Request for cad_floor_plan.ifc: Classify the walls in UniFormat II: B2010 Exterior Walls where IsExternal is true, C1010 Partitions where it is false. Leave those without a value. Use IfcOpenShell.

First a look at what the model holds.

```python
import ifcopenshell
import ifcopenshell.util.element

model = ifcopenshell.open("cad_floor_plan.ifc")
print(model.schema)
print("classifications:", [c.Name for c in model.by_type("IfcClassification")])
values = [ifcopenshell.util.element.get_pset(e, "Pset_WallCommon", "IsExternal") for e in model.by_type("IfcWall")]
for value in (True, False, None):
    print("IsExternal", value, values.count(value))
```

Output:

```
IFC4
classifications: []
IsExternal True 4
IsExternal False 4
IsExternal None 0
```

```python
import ifcopenshell
import ifcopenshell.api.classification
import ifcopenshell.util.element

model = ifcopenshell.open("cad_floor_plan.ifc")

system = ifcopenshell.api.classification.add_classification(model, classification="UniFormat II")

walls = model.by_type("IfcWall")
external = {e: ifcopenshell.util.element.get_pset(e, "Pset_WallCommon", "IsExternal") for e in walls}
for flag, code, name in ((True, "B2010", "Exterior Walls"), (False, "C1010", "Partitions")):
    products = [e for e in walls if external[e] is flag]
    ifcopenshell.api.classification.add_reference(
        model, products=products, classification=system, identification=code, name=name
    )
    print(code, len(products))

model.write("cad_floor_plan_updated.ifc")
```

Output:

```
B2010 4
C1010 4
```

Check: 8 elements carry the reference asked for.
